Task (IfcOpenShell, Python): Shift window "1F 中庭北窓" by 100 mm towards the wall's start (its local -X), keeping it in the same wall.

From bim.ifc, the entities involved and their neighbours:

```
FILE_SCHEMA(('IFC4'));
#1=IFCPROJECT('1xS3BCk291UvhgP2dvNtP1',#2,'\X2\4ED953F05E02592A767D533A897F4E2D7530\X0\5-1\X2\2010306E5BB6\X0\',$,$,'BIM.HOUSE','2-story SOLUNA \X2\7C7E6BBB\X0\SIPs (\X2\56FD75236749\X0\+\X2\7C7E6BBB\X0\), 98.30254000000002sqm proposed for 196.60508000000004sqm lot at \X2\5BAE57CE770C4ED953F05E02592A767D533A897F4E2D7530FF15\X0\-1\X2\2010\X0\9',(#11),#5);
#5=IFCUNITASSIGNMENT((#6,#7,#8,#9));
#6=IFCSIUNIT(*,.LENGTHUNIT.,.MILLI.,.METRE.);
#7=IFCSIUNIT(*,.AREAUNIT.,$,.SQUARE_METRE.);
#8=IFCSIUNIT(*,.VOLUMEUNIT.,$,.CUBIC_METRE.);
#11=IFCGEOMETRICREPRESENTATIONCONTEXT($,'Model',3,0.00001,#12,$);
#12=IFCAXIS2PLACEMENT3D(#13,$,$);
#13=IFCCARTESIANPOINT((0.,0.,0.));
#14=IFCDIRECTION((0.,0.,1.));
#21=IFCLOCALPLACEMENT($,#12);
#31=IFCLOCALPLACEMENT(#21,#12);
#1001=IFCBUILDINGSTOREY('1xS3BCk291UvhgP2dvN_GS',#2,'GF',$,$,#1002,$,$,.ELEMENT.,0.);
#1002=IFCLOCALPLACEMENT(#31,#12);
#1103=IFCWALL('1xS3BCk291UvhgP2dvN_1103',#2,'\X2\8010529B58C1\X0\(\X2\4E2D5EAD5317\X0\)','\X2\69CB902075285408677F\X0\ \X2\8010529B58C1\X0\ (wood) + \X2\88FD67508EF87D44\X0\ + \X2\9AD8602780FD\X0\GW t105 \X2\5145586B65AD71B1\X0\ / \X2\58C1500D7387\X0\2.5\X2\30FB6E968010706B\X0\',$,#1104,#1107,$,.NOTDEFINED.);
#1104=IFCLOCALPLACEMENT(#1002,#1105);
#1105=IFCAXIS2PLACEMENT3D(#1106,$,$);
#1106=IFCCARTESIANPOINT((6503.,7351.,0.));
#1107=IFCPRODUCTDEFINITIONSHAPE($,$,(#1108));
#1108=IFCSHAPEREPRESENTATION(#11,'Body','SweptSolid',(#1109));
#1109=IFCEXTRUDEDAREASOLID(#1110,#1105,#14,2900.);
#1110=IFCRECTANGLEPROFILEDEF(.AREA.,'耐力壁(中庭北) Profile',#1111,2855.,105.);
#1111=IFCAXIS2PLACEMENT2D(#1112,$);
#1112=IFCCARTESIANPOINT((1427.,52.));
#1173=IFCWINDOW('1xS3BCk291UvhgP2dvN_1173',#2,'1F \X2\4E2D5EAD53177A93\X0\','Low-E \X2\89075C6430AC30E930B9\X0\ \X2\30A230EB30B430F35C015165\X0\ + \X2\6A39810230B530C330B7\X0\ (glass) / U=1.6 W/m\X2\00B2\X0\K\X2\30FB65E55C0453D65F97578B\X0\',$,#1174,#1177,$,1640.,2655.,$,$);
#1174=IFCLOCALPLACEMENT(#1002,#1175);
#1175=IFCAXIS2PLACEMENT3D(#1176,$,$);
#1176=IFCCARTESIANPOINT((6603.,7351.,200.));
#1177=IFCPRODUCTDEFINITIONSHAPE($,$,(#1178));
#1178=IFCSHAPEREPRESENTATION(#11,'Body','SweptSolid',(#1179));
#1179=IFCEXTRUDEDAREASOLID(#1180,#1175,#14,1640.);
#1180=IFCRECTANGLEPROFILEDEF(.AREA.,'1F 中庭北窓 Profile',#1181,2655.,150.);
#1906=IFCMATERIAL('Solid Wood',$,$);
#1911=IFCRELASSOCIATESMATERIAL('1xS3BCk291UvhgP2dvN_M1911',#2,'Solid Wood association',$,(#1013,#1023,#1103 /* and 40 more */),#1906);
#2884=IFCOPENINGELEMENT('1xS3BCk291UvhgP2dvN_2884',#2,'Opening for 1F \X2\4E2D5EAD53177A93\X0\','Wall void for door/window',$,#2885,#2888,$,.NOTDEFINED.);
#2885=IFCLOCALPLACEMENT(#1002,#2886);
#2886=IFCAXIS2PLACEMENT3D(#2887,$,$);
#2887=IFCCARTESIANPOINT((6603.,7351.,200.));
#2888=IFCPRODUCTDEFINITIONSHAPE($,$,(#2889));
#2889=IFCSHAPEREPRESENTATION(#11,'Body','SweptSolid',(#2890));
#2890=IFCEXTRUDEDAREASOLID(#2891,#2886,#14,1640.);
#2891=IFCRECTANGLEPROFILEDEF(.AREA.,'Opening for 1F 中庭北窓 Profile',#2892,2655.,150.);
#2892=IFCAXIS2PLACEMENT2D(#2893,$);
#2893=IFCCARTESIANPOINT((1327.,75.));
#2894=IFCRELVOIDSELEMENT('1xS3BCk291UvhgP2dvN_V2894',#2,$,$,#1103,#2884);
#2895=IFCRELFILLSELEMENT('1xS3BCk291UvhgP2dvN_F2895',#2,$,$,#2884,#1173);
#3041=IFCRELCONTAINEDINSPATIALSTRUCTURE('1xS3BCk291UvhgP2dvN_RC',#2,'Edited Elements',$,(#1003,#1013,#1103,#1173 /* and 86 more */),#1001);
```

```python
import ifcopenshell
import ifcopenshell.api.geometry
import ifcopenshell.util.placement

model = ifcopenshell.open("bim.ifc")

window = model.by_guid("1xS3BCk291UvhgP2dvN_1173")
opening = window.FillsVoids[0].RelatingOpeningElement
wall = opening.VoidsElements[0].RelatingBuildingElement

wall_matrix = ifcopenshell.util.placement.get_local_placement(wall.ObjectPlacement)
shift = wall_matrix[:3, 0] * -100.0
before = ifcopenshell.util.placement.get_local_placement(window.ObjectPlacement)[:3, 3].copy()

# The window is not placed relative to its opening, so move both.
for product in (opening, window):
    matrix = ifcopenshell.util.placement.get_local_placement(product.ObjectPlacement)
    matrix[:3, 3] += shift
    ifcopenshell.api.geometry.edit_object_placement(model, product=product, matrix=matrix, is_si=False)

after = ifcopenshell.util.placement.get_local_placement(window.ObjectPlacement)[:3, 3]
print("window moved by", (after - before).round(3) + 0.0)

model.write("bim_updated.ifc")
```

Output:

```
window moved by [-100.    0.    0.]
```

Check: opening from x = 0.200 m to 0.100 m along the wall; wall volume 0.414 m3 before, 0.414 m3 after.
